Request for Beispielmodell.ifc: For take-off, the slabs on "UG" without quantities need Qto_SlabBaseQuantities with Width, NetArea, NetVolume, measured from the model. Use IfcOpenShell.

First a look at what the model holds.

```python
import ifcopenshell
import ifcopenshell.util.element
import ifcopenshell.util.unit

model = ifcopenshell.open("Beispielmodell.ifc")
print(model.schema)
for unit_type in ("LENGTHUNIT", "AREAUNIT", "VOLUMEUNIT"):
    print(unit_type, ifcopenshell.util.unit.calculate_unit_scale(model, unit_type))
storey = next(s for s in model.by_type("IfcBuildingStorey") if s.Name == "UG")
slabs = [e for e in ifcopenshell.util.element.get_decomposition(storey) if e.is_a("IfcSlab")]
for e in sorted(slabs, key=lambda e: e.id()):
    print(e.id(), e.is_a(), e.Name, list(ifcopenshell.util.element.get_psets(e, qtos_only=True)), sep=" | ")
```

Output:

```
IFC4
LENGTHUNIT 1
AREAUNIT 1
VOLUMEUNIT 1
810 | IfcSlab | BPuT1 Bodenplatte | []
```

```python
import ifcopenshell
import ifcopenshell.api.pset
import ifcopenshell.geom
import ifcopenshell.util.element
import ifcopenshell.util.shape
import ifcopenshell.util.unit

model = ifcopenshell.open("Beispielmodell.ifc")
unit_scale = ifcopenshell.util.unit.calculate_unit_scale(model)
area_scale = ifcopenshell.util.unit.calculate_unit_scale(model, "AREAUNIT")
volume_scale = ifcopenshell.util.unit.calculate_unit_scale(model, "VOLUMEUNIT")
settings = ifcopenshell.geom.settings()

storey = next(s for s in model.by_type("IfcBuildingStorey") if s.Name == "UG")
slabs = [e for e in ifcopenshell.util.element.get_decomposition(storey) if e.is_a("IfcSlab")]

for e in sorted(slabs, key=lambda e: e.id()):
    if ifcopenshell.util.element.get_psets(e, qtos_only=True, should_inherit=False):
        continue
    # Geometry comes back in metres, in the element's own axes.
    shape = ifcopenshell.geom.create_shape(settings, e)
    values = {
        "Width": ifcopenshell.util.shape.get_z(shape.geometry) / unit_scale,
        "NetArea": ifcopenshell.util.shape.get_footprint_area(shape.geometry) / area_scale,
        "NetVolume": ifcopenshell.util.shape.get_volume(shape.geometry) / volume_scale,
    }
    qto = ifcopenshell.api.pset.add_qto(model, product=e, name="Qto_SlabBaseQuantities")
    ifcopenshell.api.pset.edit_qto(model, qto=qto, properties=values)
    print(e.id(), {k: round(v, 3) for k, v in values.items()})

model.write("Beispielmodell_v2.ifc")
```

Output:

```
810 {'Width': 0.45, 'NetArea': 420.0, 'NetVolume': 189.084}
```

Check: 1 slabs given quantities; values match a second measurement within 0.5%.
